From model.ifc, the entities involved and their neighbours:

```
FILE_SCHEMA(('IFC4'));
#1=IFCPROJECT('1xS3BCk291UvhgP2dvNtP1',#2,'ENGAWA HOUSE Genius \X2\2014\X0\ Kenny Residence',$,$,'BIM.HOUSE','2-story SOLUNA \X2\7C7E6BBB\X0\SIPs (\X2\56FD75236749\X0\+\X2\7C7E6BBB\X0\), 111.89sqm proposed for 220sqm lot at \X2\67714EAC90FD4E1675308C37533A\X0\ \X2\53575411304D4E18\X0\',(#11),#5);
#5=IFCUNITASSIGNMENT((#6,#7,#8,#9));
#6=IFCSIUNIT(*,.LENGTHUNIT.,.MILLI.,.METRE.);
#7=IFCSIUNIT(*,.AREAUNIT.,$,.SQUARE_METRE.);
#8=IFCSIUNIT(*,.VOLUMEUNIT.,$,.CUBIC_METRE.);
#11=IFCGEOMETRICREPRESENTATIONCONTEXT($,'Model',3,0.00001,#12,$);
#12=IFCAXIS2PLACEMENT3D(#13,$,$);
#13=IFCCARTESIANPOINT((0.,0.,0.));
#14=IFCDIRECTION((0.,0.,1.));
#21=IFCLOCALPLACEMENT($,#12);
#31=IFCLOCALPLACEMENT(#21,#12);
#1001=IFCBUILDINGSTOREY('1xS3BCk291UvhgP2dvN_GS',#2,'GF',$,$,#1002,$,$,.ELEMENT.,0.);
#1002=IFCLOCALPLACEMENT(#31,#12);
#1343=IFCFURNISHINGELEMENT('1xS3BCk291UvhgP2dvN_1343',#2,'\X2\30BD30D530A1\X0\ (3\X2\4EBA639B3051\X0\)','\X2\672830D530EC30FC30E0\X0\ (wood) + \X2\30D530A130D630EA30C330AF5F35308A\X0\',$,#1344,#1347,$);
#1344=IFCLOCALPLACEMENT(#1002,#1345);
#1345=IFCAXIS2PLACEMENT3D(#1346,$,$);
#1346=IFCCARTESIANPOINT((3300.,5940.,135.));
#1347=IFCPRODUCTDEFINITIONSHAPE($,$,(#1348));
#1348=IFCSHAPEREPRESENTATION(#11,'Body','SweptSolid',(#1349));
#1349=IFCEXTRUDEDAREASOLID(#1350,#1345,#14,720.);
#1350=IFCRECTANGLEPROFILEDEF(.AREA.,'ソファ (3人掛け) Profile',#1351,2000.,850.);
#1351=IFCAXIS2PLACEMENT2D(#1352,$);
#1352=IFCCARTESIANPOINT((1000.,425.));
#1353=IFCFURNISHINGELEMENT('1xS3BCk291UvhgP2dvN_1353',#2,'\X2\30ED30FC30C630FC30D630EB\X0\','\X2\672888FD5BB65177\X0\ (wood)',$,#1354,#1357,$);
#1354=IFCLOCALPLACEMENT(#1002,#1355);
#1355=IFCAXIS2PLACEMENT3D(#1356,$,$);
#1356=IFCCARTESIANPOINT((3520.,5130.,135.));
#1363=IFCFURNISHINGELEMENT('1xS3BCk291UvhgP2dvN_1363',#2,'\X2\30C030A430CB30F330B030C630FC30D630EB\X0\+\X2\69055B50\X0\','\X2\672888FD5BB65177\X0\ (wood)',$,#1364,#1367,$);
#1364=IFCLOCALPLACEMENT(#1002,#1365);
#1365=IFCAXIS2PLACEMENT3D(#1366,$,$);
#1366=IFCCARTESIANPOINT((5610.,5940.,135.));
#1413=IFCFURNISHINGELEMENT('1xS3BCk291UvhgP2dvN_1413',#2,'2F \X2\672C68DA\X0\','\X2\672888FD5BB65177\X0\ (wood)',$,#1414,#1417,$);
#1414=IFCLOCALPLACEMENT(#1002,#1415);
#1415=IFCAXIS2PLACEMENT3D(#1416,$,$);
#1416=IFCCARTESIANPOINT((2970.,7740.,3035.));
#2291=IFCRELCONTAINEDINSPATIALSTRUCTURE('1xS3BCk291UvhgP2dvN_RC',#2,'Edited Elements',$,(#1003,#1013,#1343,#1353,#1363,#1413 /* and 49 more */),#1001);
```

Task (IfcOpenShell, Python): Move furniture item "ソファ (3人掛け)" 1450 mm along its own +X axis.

```python
import ifcopenshell
import ifcopenshell.api.geometry
import ifcopenshell.util.placement
import ifcopenshell.util.unit

model = ifcopenshell.open("model.ifc")
unit_scale = ifcopenshell.util.unit.calculate_unit_scale(model)

item = model.by_guid("1xS3BCk291UvhgP2dvN_1343")
matrix = ifcopenshell.util.placement.get_local_placement(item.ObjectPlacement)
matrix[:3, 3] += matrix[:3, 0] * 1.45 / unit_scale
ifcopenshell.api.geometry.edit_object_placement(model, product=item, matrix=matrix, is_si=False)

print(ifcopenshell.util.placement.get_local_placement(item.ObjectPlacement).round(3) + 0.0)

model.write("model_v2.ifc")
```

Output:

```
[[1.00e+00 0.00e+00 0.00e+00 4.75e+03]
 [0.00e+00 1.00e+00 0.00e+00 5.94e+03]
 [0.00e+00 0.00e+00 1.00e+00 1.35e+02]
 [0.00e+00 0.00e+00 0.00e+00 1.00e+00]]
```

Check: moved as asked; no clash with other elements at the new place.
